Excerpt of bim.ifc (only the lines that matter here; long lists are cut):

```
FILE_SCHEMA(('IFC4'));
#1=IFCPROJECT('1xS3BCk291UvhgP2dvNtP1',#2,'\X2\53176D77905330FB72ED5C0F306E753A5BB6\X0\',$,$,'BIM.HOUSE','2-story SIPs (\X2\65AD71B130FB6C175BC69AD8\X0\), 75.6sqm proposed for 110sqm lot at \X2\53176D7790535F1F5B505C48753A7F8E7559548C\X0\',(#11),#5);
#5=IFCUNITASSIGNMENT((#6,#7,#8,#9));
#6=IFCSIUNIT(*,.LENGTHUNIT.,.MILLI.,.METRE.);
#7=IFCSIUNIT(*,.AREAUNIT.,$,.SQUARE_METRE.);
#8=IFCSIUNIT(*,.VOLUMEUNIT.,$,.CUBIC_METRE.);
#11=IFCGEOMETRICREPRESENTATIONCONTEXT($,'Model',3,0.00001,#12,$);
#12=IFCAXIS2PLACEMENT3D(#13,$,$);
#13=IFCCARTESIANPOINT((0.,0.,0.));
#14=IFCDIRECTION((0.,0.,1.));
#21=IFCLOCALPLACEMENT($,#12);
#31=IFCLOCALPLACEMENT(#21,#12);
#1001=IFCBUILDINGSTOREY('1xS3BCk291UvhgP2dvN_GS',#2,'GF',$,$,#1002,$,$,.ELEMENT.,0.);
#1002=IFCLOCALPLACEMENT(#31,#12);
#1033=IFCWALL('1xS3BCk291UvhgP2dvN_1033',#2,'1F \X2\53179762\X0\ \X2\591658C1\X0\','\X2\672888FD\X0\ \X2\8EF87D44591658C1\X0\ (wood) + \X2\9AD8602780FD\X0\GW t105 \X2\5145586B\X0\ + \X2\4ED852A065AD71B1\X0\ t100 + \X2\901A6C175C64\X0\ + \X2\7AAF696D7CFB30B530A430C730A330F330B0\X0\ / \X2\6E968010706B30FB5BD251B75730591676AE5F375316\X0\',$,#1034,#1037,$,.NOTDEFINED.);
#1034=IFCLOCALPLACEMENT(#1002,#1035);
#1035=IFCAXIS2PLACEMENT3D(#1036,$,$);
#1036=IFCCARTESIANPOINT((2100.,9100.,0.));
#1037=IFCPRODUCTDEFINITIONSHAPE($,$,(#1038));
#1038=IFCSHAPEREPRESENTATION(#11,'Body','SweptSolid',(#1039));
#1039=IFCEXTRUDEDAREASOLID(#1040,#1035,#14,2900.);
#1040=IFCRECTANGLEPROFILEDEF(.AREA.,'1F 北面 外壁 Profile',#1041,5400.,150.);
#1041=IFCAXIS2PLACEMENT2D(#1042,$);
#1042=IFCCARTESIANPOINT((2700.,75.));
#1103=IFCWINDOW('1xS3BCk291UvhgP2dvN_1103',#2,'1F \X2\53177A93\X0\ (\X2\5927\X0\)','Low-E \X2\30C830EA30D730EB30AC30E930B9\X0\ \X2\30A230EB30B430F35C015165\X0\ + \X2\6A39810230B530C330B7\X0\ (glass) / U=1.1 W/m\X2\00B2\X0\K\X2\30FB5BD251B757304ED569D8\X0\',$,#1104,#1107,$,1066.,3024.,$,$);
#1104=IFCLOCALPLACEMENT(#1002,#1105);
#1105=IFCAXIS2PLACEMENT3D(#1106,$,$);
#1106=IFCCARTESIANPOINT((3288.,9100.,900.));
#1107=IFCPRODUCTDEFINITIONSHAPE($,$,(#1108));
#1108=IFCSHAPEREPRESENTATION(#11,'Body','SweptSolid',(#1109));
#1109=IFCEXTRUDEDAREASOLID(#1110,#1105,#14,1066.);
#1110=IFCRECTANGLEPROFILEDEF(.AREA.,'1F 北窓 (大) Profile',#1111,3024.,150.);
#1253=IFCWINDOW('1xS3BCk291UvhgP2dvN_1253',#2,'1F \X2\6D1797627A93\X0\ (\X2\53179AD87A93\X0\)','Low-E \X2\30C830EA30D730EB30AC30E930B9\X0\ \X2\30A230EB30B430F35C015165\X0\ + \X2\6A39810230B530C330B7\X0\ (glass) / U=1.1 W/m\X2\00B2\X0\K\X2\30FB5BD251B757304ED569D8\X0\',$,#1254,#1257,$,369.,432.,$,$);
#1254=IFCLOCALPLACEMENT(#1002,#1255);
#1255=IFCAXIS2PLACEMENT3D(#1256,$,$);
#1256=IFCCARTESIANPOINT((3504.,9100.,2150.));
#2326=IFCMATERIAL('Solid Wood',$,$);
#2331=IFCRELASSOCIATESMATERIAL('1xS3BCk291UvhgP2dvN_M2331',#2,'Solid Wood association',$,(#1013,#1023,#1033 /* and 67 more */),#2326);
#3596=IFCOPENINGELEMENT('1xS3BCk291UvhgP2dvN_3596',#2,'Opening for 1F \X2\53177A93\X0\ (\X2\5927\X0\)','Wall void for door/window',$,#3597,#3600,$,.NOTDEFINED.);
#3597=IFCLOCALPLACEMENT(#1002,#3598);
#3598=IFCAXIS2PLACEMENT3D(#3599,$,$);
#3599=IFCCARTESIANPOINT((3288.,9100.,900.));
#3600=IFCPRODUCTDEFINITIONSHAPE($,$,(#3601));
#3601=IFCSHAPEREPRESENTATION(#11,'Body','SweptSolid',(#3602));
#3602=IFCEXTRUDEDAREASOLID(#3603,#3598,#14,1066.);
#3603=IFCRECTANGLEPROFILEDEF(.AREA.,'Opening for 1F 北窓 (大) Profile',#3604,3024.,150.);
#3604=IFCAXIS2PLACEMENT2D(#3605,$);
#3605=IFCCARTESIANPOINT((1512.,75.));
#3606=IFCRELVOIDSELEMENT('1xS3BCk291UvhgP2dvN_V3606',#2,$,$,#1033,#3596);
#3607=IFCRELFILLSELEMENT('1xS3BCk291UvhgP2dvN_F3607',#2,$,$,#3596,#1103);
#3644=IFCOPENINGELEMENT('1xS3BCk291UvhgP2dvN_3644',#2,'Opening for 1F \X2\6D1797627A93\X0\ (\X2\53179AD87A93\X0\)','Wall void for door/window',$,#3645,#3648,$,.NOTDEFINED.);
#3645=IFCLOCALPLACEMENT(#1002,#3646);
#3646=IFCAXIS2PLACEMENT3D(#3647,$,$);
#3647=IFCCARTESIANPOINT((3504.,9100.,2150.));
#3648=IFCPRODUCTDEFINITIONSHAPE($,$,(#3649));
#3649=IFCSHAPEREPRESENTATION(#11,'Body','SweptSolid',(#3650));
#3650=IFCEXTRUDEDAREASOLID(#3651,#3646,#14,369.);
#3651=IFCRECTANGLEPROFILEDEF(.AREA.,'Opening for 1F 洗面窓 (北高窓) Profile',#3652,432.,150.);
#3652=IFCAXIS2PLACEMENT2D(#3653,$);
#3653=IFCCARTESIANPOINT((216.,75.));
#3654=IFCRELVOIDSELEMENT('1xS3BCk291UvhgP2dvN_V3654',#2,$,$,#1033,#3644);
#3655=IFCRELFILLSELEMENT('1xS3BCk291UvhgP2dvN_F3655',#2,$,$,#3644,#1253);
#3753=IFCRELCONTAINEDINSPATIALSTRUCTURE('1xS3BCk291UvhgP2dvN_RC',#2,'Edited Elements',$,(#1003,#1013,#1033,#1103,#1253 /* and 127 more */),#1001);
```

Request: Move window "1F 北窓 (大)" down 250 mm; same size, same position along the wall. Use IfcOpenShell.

```python
import numpy as np
import ifcopenshell
import ifcopenshell.api.geometry
import ifcopenshell.util.placement
import ifcopenshell.util.unit

model = ifcopenshell.open("bim.ifc")
unit_scale = ifcopenshell.util.unit.calculate_unit_scale(model)

window = model.by_guid("1xS3BCk291UvhgP2dvN_1103")
opening = window.FillsVoids[0].RelatingOpeningElement
dz = -250.0

shift = np.array([0.0, 0.0, dz])
# The window is not placed relative to its opening, so move both.
for product in (opening, window):
    matrix = ifcopenshell.util.placement.get_local_placement(product.ObjectPlacement)
    matrix[:3, 3] += shift
    ifcopenshell.api.geometry.edit_object_placement(model, product=product, matrix=matrix, is_si=False)

print(f"moved by {dz * unit_scale:+.3f} m")

model.write("bim_edited.ifc")
```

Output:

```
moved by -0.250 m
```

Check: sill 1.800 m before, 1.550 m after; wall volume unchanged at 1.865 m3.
